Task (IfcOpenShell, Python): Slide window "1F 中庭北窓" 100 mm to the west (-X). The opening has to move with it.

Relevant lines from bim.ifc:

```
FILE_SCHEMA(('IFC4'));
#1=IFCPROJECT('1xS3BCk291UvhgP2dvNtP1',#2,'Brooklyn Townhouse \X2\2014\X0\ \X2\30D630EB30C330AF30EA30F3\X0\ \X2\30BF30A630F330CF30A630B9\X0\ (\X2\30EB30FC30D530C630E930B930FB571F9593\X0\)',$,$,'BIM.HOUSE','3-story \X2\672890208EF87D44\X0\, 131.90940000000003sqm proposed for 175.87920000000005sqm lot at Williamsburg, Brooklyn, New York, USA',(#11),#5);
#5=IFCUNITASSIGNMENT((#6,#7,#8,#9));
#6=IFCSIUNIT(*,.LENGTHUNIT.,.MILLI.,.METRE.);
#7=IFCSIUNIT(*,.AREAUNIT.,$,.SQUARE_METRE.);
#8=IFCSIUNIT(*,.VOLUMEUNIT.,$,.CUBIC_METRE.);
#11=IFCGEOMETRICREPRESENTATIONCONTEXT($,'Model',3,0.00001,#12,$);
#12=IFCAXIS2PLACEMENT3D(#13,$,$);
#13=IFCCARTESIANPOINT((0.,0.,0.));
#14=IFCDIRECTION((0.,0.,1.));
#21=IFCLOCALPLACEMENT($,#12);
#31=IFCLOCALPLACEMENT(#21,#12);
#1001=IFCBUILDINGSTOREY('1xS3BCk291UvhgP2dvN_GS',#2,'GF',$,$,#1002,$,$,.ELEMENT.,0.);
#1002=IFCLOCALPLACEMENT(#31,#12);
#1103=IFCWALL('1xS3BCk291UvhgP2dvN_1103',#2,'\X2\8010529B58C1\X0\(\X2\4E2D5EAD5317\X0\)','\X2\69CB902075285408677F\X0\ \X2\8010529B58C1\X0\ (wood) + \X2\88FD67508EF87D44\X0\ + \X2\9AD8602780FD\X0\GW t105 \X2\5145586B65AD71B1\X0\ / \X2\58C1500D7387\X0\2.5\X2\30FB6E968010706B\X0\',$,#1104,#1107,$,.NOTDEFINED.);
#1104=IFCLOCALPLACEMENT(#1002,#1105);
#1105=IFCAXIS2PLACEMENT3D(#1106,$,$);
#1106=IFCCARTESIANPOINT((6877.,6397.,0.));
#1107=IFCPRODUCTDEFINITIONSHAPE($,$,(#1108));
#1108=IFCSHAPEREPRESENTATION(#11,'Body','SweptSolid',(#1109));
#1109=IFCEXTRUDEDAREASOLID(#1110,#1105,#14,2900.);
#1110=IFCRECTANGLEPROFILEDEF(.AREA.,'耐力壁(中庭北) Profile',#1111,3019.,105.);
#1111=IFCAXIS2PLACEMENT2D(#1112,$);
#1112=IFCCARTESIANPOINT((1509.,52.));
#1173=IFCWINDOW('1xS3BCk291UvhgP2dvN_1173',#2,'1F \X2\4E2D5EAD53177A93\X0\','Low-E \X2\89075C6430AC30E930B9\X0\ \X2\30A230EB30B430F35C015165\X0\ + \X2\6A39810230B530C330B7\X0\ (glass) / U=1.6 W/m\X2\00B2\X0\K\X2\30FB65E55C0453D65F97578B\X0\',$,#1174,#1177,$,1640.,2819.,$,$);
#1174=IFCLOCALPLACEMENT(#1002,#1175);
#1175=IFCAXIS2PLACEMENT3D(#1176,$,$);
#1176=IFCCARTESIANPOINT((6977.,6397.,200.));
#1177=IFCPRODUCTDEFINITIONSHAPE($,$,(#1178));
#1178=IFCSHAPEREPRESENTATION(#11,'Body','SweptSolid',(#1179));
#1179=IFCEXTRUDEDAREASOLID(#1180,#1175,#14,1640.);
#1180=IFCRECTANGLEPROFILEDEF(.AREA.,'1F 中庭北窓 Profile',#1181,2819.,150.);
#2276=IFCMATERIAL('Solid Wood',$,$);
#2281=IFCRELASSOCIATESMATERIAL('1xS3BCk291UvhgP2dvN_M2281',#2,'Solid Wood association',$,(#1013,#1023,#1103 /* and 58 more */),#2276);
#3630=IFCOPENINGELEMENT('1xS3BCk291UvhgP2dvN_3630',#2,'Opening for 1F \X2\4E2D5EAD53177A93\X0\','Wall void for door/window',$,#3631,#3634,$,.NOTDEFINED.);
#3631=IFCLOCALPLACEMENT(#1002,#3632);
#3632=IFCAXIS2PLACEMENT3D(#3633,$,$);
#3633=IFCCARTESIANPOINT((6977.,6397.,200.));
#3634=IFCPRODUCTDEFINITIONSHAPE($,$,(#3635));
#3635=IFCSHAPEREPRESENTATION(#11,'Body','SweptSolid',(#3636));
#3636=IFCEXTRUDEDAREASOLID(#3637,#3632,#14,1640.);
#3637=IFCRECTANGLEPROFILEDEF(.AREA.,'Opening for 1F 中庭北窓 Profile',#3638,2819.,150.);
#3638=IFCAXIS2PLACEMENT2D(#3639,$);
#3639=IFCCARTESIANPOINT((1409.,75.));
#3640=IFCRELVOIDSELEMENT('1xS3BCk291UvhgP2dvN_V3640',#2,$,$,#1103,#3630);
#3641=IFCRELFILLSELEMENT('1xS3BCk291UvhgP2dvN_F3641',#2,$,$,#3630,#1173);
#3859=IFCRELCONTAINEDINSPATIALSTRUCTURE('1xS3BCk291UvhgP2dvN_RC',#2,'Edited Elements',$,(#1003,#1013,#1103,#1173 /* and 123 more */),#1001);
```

```python
import ifcopenshell
import ifcopenshell.api.geometry
import ifcopenshell.util.placement
import ifcopenshell.util.unit

model = ifcopenshell.open("bim.ifc")
unit_scale = ifcopenshell.util.unit.calculate_unit_scale(model)

window = model.by_id(1173)
opening = window.FillsVoids[0].RelatingOpeningElement
wall = opening.VoidsElements[0].RelatingBuildingElement

wall_matrix = ifcopenshell.util.placement.get_local_placement(wall.ObjectPlacement)
shift = wall_matrix[:3, 0] * -0.1 / unit_scale
before = ifcopenshell.util.placement.get_local_placement(window.ObjectPlacement)[:3, 3].copy()

# The window is not placed relative to its opening, so move both.
for product in (opening, window):
    matrix = ifcopenshell.util.placement.get_local_placement(product.ObjectPlacement)
    matrix[:3, 3] += shift
    ifcopenshell.api.geometry.edit_object_placement(model, product=product, matrix=matrix, is_si=False)

after = ifcopenshell.util.placement.get_local_placement(window.ObjectPlacement)[:3, 3]
print("window moved by", (after - before).round(3) + 0.0)

model.write("bim_rev.ifc")
```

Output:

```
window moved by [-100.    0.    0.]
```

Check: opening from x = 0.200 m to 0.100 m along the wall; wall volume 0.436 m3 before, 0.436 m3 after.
